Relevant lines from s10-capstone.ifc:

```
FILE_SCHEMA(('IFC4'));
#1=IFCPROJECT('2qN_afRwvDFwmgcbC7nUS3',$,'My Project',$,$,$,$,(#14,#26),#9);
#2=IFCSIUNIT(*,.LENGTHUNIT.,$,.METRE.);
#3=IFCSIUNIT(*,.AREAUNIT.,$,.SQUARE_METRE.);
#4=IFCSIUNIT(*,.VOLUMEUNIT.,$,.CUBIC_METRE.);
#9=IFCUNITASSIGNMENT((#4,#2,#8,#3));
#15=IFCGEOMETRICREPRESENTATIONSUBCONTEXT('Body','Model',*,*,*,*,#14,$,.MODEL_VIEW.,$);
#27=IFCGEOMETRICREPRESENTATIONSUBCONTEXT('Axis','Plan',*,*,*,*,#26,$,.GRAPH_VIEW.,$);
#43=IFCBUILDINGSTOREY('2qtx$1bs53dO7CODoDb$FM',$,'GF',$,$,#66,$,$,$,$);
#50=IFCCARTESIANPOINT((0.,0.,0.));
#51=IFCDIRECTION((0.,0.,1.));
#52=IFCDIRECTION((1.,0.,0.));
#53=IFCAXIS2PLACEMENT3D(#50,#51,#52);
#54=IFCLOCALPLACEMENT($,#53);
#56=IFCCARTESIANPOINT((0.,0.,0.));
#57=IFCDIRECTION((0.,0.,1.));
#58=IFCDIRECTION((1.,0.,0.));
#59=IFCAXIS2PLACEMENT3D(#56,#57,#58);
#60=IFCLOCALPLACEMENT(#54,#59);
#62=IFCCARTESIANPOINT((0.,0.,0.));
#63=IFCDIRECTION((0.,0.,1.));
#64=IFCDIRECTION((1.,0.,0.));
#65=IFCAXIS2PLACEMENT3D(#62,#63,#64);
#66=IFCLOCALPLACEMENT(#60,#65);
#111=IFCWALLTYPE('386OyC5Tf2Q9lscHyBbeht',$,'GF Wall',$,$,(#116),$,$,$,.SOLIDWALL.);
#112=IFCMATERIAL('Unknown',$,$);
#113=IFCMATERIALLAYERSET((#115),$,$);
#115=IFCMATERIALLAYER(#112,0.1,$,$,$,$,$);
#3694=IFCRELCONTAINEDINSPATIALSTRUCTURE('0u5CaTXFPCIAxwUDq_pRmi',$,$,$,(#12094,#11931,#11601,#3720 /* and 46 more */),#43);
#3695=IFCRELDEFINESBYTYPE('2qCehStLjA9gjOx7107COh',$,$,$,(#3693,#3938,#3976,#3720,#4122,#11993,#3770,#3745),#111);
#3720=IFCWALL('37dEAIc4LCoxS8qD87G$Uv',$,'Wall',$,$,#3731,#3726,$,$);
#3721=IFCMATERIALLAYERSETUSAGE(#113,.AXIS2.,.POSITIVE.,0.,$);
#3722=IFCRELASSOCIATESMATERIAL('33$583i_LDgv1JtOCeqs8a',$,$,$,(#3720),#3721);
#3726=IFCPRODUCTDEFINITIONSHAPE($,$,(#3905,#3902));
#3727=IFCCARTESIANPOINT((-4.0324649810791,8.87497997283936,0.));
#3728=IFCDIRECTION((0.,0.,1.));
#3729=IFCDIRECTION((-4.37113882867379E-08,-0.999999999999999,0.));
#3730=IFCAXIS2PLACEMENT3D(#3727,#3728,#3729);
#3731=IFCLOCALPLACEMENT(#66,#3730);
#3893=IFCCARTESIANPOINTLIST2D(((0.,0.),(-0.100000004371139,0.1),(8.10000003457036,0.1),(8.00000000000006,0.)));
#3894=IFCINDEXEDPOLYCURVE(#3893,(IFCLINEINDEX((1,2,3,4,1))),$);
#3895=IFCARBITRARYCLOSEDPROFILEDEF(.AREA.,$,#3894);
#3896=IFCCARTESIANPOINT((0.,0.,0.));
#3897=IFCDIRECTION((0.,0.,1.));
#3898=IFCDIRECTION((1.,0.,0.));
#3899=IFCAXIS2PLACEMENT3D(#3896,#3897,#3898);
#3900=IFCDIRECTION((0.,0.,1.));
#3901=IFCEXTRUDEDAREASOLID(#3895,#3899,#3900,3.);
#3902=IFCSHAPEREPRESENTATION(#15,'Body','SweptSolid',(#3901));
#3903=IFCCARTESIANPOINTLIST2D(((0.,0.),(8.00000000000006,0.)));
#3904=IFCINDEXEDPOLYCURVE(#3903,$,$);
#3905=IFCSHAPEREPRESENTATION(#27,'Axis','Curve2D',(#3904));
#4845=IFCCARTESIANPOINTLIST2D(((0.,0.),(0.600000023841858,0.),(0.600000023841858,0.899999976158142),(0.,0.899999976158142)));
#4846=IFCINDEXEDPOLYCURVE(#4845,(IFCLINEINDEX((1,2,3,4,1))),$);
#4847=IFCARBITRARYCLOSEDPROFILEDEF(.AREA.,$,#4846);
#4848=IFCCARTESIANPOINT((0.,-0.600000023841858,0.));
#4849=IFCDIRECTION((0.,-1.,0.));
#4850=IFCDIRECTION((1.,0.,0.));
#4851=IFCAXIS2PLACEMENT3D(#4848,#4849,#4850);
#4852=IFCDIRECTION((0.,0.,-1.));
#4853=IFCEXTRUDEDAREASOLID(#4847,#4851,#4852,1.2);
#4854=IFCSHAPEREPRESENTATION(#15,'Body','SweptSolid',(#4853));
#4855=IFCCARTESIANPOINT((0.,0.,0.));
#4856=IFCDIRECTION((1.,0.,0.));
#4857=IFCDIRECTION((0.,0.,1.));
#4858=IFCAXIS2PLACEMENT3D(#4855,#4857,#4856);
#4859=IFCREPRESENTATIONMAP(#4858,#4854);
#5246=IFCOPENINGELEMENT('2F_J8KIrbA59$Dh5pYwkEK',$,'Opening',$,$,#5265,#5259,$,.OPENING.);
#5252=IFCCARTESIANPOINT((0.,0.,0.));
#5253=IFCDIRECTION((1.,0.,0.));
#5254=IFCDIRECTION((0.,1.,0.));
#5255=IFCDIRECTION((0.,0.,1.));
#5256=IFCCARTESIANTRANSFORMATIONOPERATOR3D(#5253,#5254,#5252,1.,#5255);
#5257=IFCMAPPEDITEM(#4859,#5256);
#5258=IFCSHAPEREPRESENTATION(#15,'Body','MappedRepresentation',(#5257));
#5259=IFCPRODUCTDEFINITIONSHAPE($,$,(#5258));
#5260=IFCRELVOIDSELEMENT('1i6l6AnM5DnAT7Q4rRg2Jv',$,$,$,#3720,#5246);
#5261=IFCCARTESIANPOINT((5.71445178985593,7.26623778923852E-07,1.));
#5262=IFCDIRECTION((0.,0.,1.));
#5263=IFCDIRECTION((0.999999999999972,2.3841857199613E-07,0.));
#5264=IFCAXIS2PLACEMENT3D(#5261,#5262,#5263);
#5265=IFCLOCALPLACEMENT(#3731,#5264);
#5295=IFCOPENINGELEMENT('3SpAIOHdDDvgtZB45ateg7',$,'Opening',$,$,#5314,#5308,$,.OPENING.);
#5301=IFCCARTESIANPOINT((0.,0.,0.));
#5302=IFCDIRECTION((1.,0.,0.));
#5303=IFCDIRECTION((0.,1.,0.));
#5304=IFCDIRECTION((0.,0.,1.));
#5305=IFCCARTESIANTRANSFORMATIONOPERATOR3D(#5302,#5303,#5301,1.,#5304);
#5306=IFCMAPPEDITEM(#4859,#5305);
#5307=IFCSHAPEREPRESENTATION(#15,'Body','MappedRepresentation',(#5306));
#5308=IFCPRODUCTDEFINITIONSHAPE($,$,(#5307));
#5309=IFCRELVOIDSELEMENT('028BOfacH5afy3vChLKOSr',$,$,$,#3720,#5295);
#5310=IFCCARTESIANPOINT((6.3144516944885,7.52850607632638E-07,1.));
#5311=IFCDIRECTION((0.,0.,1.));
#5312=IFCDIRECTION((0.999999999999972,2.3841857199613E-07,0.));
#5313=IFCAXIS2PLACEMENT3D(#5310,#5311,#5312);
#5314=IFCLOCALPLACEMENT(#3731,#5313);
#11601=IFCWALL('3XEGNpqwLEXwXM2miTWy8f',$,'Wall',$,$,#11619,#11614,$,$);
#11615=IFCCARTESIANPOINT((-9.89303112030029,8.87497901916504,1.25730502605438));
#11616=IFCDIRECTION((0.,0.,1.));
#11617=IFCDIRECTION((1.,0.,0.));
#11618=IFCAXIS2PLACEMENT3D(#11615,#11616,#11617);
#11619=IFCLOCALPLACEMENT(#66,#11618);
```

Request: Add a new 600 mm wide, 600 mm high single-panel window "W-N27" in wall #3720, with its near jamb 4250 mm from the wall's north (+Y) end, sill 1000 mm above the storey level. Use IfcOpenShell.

```python
import numpy as np
import ifcopenshell
import ifcopenshell.api.feature
import ifcopenshell.api.geometry
import ifcopenshell.api.root
import ifcopenshell.api.spatial
import ifcopenshell.geom
import ifcopenshell.util.element
import ifcopenshell.util.placement
import ifcopenshell.util.representation
import ifcopenshell.util.shape
import ifcopenshell.util.unit

model = ifcopenshell.open("s10-capstone.ifc")
unit_scale = ifcopenshell.util.unit.calculate_unit_scale(model)
settings = ifcopenshell.geom.settings()


def volume(element):
    """Net volume in cubic metres, openings subtracted."""
    shape = ifcopenshell.geom.create_shape(settings, element)
    return ifcopenshell.util.shape.get_volume(shape.geometry)


wall = model.by_guid("37dEAIc4LCoxS8qD87G$Uv")
storey = ifcopenshell.util.element.get_container(wall, ifc_class="IfcBuildingStorey")
context = ifcopenshell.util.representation.get_context(model, "Model", "Body", "MODEL_VIEW")
before = volume(wall)

width, height, from_end, sill = 0.6, 0.6, 4.25, 1  # metres

# The wall runs along its own X axis, and the end named is its -X end.
wall_shape = ifcopenshell.geom.create_shape(settings, wall)
x, y, z = ifcopenshell.util.shape.get_vertices(wall_shape.geometry).T
start = x.min() + from_end
face, thickness = float(y.min()), float(y.max() - y.min())
wall_matrix = ifcopenshell.util.placement.get_local_placement(wall.ObjectPlacement)
level = ifcopenshell.util.placement.get_local_placement(storey.ObjectPlacement)[2, 3]


def in_wall(x, y):
    """Placement at x, y metres in the wall's axes, at sill height."""
    matrix = wall_matrix.copy()
    matrix[:, 3] = wall_matrix @ np.array([x / unit_scale, y / unit_scale, 0.0, 1.0])
    matrix[2, 3] = level + sill / unit_scale
    return matrix


# Opening: a box that overshoots both wall faces by 50 mm.
opening = ifcopenshell.api.root.create_entity(model, ifc_class="IfcOpeningElement", predefined_type="OPENING")
box = ifcopenshell.api.geometry.add_wall_representation(
    model, context=context, length=width, height=height, thickness=thickness + 0.1
)
ifcopenshell.api.geometry.assign_representation(model, product=opening, representation=box)
ifcopenshell.api.geometry.edit_object_placement(model, product=opening, matrix=in_wall(start, face - 0.05), is_si=False)
ifcopenshell.api.feature.add_feature(model, feature=opening, element=wall)

window = ifcopenshell.api.root.create_entity(model, ifc_class="IfcWindow", name="W-N27", predefined_type="WINDOW")
window.OverallWidth, window.OverallHeight = width / unit_scale, height / unit_scale
window.PartitioningType = "SINGLE_PANEL"
body = ifcopenshell.api.geometry.add_window_representation(
    model,
    context=context,
    overall_width=window.OverallWidth,
    overall_height=window.OverallHeight,
    partition_type="SINGLE_PANEL",
)
ifcopenshell.api.geometry.assign_representation(model, product=window, representation=body)
ifcopenshell.api.spatial.assign_container(model, products=[window], relating_structure=storey)
ifcopenshell.api.feature.add_filling(model, opening=opening, element=window)

# Centre the window in the wall's thickness.
ifcopenshell.api.geometry.edit_object_placement(model, product=window, matrix=in_wall(start, face), is_si=False)
window_shape = ifcopenshell.geom.create_shape(settings, window)
depth = ifcopenshell.util.shape.get_vertices(window_shape.geometry)[:, 1]
offset = face + thickness / 2 - (depth.min() + depth.max()) / 2
ifcopenshell.api.geometry.edit_object_placement(model, product=window, matrix=in_wall(start, offset), is_si=False)

after = volume(wall)

print(f"wall volume {before:.3f} -> {after:.3f} m3")

model.write("s10-capstone_edited.ifc")
```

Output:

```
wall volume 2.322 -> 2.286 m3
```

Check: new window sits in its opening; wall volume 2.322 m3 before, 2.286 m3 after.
